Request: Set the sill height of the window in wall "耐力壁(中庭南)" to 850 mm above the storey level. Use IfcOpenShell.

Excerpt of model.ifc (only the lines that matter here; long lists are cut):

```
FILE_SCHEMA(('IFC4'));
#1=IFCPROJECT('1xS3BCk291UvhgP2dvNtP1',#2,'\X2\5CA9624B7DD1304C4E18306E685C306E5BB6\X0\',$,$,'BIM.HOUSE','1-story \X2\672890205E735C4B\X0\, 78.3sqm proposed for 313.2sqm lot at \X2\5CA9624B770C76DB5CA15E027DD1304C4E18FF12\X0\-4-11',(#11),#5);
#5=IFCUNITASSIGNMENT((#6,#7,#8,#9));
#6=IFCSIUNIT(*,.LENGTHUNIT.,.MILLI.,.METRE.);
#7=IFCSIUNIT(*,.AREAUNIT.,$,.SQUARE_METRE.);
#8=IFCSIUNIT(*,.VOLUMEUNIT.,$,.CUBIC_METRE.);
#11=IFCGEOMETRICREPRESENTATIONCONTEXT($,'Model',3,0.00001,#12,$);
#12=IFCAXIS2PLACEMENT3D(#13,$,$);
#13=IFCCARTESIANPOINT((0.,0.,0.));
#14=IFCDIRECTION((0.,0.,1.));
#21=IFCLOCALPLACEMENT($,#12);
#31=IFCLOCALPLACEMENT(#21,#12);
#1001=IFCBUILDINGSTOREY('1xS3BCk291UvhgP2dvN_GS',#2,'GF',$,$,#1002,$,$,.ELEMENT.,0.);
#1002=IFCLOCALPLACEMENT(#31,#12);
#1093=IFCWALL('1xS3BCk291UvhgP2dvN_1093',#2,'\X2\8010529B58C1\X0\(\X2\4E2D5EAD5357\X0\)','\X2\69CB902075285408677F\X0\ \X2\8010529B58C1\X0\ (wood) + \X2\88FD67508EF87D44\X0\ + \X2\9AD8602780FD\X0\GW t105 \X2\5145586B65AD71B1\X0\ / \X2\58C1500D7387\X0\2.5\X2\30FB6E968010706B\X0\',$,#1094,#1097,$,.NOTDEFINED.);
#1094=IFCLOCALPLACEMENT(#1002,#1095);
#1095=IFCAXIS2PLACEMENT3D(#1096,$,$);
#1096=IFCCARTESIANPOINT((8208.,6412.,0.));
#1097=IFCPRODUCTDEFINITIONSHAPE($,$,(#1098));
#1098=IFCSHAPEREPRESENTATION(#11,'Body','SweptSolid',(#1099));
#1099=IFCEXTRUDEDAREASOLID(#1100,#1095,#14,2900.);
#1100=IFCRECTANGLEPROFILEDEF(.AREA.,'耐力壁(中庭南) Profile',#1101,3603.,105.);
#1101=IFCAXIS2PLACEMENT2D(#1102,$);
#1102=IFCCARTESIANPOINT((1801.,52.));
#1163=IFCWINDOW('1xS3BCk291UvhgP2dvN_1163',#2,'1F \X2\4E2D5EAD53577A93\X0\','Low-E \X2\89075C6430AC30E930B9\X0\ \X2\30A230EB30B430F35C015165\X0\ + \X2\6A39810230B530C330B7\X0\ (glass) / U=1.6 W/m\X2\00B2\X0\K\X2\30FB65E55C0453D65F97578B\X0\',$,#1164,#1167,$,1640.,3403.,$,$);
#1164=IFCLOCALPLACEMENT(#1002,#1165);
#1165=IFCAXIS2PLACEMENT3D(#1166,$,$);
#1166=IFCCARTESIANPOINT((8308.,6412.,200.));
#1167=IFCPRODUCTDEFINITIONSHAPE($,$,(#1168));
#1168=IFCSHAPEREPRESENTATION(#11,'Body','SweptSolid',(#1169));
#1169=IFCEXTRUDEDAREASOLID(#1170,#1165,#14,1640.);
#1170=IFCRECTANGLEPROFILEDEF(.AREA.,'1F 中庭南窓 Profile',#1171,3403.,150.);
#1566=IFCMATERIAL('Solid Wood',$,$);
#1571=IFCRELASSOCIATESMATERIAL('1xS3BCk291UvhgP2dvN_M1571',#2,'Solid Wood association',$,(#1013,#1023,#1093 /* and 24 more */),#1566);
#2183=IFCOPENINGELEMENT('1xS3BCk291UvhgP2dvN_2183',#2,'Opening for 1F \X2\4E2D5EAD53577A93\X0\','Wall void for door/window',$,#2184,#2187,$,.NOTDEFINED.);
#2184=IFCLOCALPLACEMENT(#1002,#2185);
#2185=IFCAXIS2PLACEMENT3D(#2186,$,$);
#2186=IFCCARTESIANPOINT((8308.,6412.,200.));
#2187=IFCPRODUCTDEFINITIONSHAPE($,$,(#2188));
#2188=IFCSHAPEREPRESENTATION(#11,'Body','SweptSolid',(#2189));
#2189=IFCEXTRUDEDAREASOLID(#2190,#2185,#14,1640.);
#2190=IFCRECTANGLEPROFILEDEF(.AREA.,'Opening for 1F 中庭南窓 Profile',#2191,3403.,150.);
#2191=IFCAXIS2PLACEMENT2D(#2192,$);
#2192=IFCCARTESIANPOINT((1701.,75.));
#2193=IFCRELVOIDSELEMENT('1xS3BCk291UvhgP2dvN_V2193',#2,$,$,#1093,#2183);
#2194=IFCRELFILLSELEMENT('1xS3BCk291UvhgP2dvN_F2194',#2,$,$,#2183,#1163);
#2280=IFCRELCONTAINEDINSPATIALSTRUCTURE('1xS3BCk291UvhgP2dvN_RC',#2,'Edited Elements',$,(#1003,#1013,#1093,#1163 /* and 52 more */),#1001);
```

```python
import numpy as np
import ifcopenshell
import ifcopenshell.api.geometry
import ifcopenshell.geom
import ifcopenshell.util.element
import ifcopenshell.util.placement
import ifcopenshell.util.shape
import ifcopenshell.util.unit

model = ifcopenshell.open("model.ifc")
unit_scale = ifcopenshell.util.unit.calculate_unit_scale(model)

window = model.by_guid("1xS3BCk291UvhgP2dvN_1163")
opening = window.FillsVoids[0].RelatingOpeningElement
storey = ifcopenshell.util.element.get_container(window, ifc_class="IfcBuildingStorey")
level = ifcopenshell.util.placement.get_local_placement(storey.ObjectPlacement)[2, 3]

# The opening's origin need not be at the sill, so measure its lowest point.
shape = ifcopenshell.geom.create_shape(ifcopenshell.geom.settings(), opening)
bottom = ifcopenshell.util.shape.get_shape_bottom_elevation(shape, shape.geometry) / unit_scale
dz = level + 0.85 / unit_scale - bottom

shift = np.array([0.0, 0.0, dz])
# The window is not placed relative to its opening, so move both.
for product in (opening, window):
    matrix = ifcopenshell.util.placement.get_local_placement(product.ObjectPlacement)
    matrix[:3, 3] += shift
    ifcopenshell.api.geometry.edit_object_placement(model, product=product, matrix=matrix, is_si=False)

print(f"moved by {dz * unit_scale:+.3f} m")

model.write("model_rev.ifc")
```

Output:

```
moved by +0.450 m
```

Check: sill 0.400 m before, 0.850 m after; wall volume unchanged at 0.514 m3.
